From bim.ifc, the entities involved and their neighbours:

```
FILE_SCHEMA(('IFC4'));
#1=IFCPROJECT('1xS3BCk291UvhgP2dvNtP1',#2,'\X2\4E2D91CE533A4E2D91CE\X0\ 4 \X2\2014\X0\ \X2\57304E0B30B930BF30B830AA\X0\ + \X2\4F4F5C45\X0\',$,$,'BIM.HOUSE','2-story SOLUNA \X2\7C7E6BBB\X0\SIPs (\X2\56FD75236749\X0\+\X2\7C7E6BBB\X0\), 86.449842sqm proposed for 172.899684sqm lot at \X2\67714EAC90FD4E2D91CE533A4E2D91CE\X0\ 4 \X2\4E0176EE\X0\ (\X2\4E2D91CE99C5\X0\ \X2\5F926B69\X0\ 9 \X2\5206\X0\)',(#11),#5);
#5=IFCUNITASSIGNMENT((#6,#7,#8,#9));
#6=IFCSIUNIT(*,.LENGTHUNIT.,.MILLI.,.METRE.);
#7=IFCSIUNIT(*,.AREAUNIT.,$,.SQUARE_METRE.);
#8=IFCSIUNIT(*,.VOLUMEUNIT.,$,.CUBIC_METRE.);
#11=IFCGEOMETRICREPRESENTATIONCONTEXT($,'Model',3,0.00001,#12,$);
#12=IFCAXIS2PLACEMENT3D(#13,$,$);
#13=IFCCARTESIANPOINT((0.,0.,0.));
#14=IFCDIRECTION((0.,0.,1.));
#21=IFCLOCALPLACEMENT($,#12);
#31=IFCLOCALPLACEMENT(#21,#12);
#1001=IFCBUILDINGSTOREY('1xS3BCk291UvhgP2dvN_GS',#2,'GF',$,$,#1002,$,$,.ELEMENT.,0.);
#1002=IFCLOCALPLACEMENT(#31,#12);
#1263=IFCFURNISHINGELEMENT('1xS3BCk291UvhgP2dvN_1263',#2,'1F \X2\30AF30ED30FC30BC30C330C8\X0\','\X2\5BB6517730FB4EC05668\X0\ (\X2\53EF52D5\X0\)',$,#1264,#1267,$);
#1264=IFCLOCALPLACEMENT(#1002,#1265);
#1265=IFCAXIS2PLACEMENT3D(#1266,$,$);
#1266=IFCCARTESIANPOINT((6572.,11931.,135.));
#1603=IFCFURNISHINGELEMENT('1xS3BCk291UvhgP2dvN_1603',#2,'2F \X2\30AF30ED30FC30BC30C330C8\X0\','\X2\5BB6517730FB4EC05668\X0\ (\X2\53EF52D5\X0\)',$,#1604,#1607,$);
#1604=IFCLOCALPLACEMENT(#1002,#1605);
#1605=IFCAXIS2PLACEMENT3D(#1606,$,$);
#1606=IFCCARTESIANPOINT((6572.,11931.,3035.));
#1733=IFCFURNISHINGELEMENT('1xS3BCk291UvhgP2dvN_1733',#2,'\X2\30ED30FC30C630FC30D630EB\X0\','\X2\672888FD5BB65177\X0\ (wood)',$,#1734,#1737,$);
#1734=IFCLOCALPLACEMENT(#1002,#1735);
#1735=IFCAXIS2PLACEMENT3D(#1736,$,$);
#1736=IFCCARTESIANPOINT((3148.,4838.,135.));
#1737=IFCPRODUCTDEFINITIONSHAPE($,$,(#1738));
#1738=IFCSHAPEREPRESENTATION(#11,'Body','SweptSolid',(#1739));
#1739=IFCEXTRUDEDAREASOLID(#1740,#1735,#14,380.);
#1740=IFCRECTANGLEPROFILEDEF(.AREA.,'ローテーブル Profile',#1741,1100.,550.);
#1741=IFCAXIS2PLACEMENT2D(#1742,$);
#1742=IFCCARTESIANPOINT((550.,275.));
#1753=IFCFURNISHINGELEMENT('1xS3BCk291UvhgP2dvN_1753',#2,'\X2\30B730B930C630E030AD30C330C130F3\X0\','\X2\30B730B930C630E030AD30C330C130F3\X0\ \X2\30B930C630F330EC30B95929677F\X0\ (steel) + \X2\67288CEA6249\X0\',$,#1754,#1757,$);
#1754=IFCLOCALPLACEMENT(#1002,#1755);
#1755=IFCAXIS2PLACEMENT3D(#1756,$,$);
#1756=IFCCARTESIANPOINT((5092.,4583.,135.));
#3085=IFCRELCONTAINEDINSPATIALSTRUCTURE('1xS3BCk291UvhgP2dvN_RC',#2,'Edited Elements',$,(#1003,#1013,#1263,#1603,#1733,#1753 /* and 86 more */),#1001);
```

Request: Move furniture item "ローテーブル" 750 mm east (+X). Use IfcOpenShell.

```python
import ifcopenshell
import ifcopenshell.api.geometry
import ifcopenshell.util.placement
import ifcopenshell.util.unit

model = ifcopenshell.open("bim.ifc")
unit_scale = ifcopenshell.util.unit.calculate_unit_scale(model)

item = model.by_guid("1xS3BCk291UvhgP2dvN_1733")
matrix = ifcopenshell.util.placement.get_local_placement(item.ObjectPlacement)
matrix[0, 3] += 0.75 / unit_scale
ifcopenshell.api.geometry.edit_object_placement(model, product=item, matrix=matrix, is_si=False)

print(ifcopenshell.util.placement.get_local_placement(item.ObjectPlacement).round(3) + 0.0)

model.write("bim-out.ifc")
```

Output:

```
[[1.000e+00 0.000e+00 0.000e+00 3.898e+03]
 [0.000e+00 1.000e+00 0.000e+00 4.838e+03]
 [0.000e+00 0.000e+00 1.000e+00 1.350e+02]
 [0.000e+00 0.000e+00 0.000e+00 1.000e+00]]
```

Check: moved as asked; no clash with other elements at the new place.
